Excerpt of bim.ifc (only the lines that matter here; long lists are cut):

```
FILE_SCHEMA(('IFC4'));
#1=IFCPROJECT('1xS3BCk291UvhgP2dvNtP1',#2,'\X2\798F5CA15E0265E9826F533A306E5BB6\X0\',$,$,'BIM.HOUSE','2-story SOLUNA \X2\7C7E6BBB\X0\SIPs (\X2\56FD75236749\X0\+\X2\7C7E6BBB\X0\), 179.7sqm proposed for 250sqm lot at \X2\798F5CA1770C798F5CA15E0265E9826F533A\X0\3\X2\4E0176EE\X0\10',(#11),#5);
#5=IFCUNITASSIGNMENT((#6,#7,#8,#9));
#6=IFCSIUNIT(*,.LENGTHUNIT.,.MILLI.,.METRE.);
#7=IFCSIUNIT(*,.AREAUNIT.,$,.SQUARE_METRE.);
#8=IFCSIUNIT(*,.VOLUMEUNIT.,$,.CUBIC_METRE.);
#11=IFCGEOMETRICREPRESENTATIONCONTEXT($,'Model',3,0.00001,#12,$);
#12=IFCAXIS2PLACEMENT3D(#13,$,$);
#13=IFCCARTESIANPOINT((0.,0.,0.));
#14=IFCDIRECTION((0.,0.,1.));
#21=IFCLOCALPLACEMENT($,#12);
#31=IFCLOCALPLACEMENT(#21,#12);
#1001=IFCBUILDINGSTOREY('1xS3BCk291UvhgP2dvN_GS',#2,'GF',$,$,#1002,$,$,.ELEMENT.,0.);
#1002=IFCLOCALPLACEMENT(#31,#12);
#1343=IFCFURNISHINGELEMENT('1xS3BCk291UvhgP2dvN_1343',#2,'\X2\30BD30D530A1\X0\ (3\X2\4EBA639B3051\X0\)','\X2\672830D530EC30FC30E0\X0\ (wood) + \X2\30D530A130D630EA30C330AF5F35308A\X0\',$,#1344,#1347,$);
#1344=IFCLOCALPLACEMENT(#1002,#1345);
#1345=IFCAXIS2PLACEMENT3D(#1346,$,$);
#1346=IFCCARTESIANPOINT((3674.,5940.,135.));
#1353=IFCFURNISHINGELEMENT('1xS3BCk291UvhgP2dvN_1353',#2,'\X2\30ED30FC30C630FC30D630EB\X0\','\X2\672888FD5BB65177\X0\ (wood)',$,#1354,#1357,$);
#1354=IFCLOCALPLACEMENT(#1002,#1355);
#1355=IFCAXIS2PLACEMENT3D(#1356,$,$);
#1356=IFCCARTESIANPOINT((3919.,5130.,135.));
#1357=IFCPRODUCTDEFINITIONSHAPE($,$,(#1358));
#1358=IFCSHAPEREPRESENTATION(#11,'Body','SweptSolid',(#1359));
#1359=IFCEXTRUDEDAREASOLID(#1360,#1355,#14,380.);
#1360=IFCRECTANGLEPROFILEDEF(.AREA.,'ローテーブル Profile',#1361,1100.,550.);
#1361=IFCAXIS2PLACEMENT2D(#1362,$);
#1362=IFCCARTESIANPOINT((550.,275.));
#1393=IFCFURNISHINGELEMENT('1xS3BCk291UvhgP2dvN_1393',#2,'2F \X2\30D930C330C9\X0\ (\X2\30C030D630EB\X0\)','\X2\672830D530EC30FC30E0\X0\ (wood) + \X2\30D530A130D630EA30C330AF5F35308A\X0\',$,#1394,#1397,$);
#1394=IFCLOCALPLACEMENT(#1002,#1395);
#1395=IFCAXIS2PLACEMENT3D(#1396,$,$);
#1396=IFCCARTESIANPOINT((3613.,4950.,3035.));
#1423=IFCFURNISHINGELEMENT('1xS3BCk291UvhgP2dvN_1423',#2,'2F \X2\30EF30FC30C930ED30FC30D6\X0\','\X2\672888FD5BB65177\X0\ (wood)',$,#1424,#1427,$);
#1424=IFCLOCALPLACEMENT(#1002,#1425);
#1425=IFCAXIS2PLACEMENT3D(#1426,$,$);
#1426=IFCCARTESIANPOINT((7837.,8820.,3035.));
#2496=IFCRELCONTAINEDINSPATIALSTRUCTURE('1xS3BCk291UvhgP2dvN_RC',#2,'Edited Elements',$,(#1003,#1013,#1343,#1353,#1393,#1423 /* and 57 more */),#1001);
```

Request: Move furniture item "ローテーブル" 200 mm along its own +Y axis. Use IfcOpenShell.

```python
import ifcopenshell
import ifcopenshell.api.geometry
import ifcopenshell.util.placement

model = ifcopenshell.open("bim.ifc")

item = model.by_guid("1xS3BCk291UvhgP2dvN_1353")
matrix = ifcopenshell.util.placement.get_local_placement(item.ObjectPlacement)
matrix[:3, 3] += matrix[:3, 1] * 200.0
ifcopenshell.api.geometry.edit_object_placement(model, product=item, matrix=matrix, is_si=False)

print(ifcopenshell.util.placement.get_local_placement(item.ObjectPlacement).round(3) + 0.0)

model.write("bim_rev.ifc")
```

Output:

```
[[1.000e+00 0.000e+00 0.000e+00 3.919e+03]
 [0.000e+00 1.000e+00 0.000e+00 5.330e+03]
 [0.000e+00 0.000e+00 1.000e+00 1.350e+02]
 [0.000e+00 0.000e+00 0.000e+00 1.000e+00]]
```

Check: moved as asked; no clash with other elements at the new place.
